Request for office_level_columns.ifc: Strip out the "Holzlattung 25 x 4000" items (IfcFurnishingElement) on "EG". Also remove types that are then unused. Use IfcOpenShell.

First a look at what the model holds.

```python
import ifcopenshell
import ifcopenshell.util.element

model = ifcopenshell.open("office_level_columns.ifc")
print(model.schema)
storey = next(s for s in model.by_type("IfcBuildingStorey") if s.Name == "EG")
furniture = [e for e in ifcopenshell.util.element.get_decomposition(storey) if e.is_a("IfcFurnishingElement")]
seen = {}
for e in furniture:
    element_type = ifcopenshell.util.element.get_type(e)
    name = element_type.Name if element_type not in (None, e) else None
    seen[name] = seen.get(name, 0) + 1
for name, count in sorted(seen.items(), key=str):
    print(count, "x", name)
```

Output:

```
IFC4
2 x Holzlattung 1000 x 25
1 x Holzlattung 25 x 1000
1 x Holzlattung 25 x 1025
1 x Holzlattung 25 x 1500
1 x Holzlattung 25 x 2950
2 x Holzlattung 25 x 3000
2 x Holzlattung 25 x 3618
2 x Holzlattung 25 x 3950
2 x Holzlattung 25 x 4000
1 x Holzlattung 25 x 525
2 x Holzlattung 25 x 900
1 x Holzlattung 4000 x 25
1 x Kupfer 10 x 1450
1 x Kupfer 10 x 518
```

```python
import ifcopenshell
import ifcopenshell.api.root
import ifcopenshell.util.element

model = ifcopenshell.open("office_level_columns.ifc")

storey = next(s for s in model.by_type("IfcBuildingStorey") if s.Name == "EG")
furniture = [e for e in ifcopenshell.util.element.get_decomposition(storey) if e.is_a("IfcFurnishingElement")]
targets = [e for e in furniture if (t := ifcopenshell.util.element.get_type(e)) not in (None, e) and t.Name == "Holzlattung 25 x 4000"]
types = {ifcopenshell.util.element.get_type(e) for e in targets} - {None, *targets}

for e in targets:
    ifcopenshell.api.root.remove_product(model, product=e)
print(len(targets), "removed")

unused = [t for t in types if not ifcopenshell.util.element.get_types(t)]
for t in unused:
    ifcopenshell.api.root.remove_product(model, product=t)
print(len(unused), "unused types removed")

model.write("office_level_columns-out.ifc")
```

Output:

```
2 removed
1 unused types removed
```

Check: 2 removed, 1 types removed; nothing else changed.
